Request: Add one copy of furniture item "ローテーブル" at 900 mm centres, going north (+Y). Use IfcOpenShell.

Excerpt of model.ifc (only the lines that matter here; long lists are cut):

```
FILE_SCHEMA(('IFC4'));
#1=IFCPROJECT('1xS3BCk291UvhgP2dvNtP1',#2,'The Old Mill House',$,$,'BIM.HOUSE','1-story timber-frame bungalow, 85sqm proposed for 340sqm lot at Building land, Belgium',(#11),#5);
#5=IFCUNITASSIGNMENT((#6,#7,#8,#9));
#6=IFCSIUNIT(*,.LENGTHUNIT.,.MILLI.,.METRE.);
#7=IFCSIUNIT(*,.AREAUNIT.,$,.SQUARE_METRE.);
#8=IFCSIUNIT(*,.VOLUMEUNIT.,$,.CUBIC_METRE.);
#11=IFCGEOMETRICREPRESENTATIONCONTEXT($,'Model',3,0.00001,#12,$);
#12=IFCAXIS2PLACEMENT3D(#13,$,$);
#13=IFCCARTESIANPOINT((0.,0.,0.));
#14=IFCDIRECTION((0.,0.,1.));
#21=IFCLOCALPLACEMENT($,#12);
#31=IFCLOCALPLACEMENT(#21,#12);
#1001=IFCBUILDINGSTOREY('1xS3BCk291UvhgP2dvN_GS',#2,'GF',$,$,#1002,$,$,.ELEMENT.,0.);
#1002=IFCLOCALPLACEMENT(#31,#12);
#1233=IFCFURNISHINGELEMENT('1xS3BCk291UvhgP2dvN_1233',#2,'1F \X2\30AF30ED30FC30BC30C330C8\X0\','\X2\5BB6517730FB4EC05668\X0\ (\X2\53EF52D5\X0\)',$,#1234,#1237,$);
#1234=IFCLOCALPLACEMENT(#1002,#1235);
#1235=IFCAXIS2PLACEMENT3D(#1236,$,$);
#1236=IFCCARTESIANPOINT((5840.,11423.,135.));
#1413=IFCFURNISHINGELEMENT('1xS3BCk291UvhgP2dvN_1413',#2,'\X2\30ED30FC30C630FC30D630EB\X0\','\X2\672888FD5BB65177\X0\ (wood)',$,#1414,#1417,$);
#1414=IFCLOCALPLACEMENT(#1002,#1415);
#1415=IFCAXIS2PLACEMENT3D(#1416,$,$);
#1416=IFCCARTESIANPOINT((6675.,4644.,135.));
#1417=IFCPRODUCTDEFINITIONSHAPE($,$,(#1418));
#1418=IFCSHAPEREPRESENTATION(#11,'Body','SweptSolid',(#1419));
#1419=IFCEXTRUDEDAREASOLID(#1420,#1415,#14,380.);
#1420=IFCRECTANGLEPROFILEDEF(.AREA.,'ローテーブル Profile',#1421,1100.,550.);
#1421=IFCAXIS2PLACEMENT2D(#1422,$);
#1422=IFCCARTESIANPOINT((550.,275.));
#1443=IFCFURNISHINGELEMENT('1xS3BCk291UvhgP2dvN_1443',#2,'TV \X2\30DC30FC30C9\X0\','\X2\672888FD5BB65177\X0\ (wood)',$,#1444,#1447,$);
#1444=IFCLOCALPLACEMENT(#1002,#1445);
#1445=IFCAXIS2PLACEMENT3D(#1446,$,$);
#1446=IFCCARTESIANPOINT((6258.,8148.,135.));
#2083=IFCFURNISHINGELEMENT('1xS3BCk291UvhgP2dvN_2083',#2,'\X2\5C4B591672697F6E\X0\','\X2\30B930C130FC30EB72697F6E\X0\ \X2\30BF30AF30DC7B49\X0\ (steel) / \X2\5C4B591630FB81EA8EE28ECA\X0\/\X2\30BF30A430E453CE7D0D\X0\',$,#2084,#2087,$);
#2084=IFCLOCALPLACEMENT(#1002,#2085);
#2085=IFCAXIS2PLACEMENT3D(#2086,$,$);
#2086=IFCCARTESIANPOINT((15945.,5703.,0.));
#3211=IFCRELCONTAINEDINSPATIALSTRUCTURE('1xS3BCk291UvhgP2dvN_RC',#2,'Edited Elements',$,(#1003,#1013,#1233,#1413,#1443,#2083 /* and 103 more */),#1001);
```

```python
import numpy as np
import ifcopenshell
import ifcopenshell.api.geometry
import ifcopenshell.api.root
import ifcopenshell.util.element
import ifcopenshell.util.placement

model = ifcopenshell.open("model.ifc")


def reuse_history(source, copy):
    """copy_class also copies each property set's owner history, people and application; keep the originals."""
    for rel in copy.IsDefinedBy:
        if rel.is_a("IfcRelDefinesByProperties") and (history := rel.RelatingPropertyDefinition.OwnerHistory):
            rel.RelatingPropertyDefinition.OwnerHistory = source.OwnerHistory
            ifcopenshell.util.element.remove_deep2(model, history)


source = model.by_id(1413)
base = ifcopenshell.util.placement.get_local_placement(source.ObjectPlacement)
step = np.array([0.0, 1.0, 0.0]) * 900.0

for i in range(1, 2):
    copy = ifcopenshell.api.root.copy_class(model, product=source)
    copy.Representation = ifcopenshell.util.element.copy_deep(
        model, source.Representation, exclude=["IfcGeometricRepresentationContext", "IfcRepresentationMap"]
    )
    reuse_history(source, copy)
    matrix = base.copy()
    matrix[:3, 3] += i * step
    print("added at", matrix[:3, 3].round(3) + 0.0)
    ifcopenshell.api.geometry.edit_object_placement(model, product=copy, matrix=matrix, is_si=False)

model.write("model_edited.ifc")
```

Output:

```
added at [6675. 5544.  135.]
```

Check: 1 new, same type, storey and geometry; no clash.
